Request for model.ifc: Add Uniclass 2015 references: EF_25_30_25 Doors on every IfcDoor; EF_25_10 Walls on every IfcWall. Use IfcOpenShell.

First a look at what the model holds.

```python
import ifcopenshell

model = ifcopenshell.open("model.ifc")
print(model.schema)
print("classifications:", [c.Name for c in model.by_type("IfcClassification")])
for ifc_class in ("IfcDoor", "IfcRoof", "IfcStair", "IfcWall", "IfcWindow"):
    print(ifc_class, len(model.by_type(ifc_class)))
```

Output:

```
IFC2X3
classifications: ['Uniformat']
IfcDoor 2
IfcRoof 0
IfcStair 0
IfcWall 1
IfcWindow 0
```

```python
import ifcopenshell
import ifcopenshell.api.classification

model = ifcopenshell.open("model.ifc")

# IFC2X3 requires Source and Edition and has no link from the project to the system.
system = model.create_entity("IfcClassification", Source="NBS", Edition="2015", Name="Uniclass 2015")

codes = {
    "IfcDoor": ("EF_25_30_25", "Doors"),
    "IfcWall": ("EF_25_10", "Walls"),
}
for ifc_class, (code, name) in codes.items():
    products = model.by_type(ifc_class)
    ifcopenshell.api.classification.add_reference(
        model, products=products, classification=system, identification=code, name=name
    )
    print(code, len(products))

model.write("model_edited.ifc")
```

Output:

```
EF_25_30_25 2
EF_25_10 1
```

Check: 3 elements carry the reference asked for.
